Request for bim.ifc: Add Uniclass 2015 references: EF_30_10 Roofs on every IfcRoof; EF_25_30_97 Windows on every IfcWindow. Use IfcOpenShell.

First a look at what the model holds.

```python
import ifcopenshell

model = ifcopenshell.open("bim.ifc")
print(model.schema)
print("classifications:", [c.Name for c in model.by_type("IfcClassification")])
for ifc_class in ("IfcDoor", "IfcRoof", "IfcStair", "IfcWall", "IfcWindow"):
    print(ifc_class, len(model.by_type(ifc_class)))
```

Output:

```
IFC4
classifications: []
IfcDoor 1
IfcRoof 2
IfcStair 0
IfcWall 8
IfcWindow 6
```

```python
import ifcopenshell
import ifcopenshell.api.classification

model = ifcopenshell.open("bim.ifc")

system = ifcopenshell.api.classification.add_classification(model, classification="Uniclass 2015")

codes = {
    "IfcRoof": ("EF_30_10", "Roofs"),
    "IfcWindow": ("EF_25_30_97", "Windows"),
}
for ifc_class, (code, name) in codes.items():
    products = model.by_type(ifc_class)
    ifcopenshell.api.classification.add_reference(
        model, products=products, classification=system, identification=code, name=name
    )
    print(code, len(products))

model.write("bim_rev.ifc")
```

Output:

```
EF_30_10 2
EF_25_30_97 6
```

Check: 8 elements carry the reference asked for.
